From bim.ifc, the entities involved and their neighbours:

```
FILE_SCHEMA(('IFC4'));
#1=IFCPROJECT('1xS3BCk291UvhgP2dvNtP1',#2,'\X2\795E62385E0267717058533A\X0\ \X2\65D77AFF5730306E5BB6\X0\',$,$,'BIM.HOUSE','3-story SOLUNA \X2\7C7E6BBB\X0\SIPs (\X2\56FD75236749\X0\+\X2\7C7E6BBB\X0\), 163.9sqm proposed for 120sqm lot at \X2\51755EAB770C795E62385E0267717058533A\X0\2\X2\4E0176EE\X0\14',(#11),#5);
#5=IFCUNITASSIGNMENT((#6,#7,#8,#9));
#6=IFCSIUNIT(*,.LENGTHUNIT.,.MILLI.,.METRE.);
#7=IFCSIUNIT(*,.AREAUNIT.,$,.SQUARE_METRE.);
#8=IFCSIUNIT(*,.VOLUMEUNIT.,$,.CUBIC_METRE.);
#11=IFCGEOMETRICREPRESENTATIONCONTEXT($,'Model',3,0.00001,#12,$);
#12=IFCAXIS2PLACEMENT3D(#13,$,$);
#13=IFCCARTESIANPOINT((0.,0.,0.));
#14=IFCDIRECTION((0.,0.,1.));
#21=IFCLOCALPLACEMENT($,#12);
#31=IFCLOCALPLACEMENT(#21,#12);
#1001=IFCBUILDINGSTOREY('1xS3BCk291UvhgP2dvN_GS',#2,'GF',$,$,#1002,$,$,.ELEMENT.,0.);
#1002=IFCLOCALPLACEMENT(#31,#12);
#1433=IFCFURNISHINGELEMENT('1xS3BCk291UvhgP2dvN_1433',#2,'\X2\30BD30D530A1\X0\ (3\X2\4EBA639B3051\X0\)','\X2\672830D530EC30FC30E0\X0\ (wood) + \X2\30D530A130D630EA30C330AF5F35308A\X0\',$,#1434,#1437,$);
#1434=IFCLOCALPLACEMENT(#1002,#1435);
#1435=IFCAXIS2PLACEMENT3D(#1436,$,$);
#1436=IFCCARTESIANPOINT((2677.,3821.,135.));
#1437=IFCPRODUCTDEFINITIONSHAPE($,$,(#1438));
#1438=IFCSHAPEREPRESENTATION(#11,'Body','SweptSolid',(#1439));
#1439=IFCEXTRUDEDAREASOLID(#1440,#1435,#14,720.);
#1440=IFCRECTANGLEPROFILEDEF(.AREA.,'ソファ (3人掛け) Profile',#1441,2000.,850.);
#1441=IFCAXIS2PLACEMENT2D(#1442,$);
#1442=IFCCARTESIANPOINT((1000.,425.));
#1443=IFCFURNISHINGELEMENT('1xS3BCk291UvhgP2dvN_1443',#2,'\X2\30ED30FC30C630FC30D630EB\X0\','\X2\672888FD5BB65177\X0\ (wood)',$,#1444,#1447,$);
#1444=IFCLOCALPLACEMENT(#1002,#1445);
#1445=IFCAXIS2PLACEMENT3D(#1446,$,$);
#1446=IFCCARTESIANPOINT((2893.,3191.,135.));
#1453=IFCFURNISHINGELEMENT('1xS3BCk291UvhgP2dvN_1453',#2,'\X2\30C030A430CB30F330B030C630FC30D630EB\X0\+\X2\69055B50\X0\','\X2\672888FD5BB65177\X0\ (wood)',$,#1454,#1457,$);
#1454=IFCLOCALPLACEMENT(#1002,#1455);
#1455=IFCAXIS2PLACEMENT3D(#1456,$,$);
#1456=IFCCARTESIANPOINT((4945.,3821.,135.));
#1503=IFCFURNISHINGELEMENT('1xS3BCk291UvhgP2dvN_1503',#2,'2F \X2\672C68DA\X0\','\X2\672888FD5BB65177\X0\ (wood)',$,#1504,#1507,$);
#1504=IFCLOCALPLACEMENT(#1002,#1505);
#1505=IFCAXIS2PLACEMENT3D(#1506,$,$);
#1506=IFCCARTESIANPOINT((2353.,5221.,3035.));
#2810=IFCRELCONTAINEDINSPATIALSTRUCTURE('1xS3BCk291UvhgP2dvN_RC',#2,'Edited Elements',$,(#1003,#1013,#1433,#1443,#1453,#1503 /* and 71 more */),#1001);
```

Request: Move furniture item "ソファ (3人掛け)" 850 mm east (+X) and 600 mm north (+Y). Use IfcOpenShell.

```python
import ifcopenshell
import ifcopenshell.api.geometry
import ifcopenshell.util.placement

model = ifcopenshell.open("bim.ifc")

item = model.by_guid("1xS3BCk291UvhgP2dvN_1433")
matrix = ifcopenshell.util.placement.get_local_placement(item.ObjectPlacement)
matrix[0, 3] += 850.0
matrix[1, 3] += 600.0
ifcopenshell.api.geometry.edit_object_placement(model, product=item, matrix=matrix, is_si=False)

print(ifcopenshell.util.placement.get_local_placement(item.ObjectPlacement).round(3) + 0.0)

model.write("bim_updated.ifc")
```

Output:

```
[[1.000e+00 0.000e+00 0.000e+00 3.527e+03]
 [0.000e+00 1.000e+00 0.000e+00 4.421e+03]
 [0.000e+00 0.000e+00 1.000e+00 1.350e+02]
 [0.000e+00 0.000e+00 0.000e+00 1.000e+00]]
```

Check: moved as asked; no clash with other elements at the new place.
